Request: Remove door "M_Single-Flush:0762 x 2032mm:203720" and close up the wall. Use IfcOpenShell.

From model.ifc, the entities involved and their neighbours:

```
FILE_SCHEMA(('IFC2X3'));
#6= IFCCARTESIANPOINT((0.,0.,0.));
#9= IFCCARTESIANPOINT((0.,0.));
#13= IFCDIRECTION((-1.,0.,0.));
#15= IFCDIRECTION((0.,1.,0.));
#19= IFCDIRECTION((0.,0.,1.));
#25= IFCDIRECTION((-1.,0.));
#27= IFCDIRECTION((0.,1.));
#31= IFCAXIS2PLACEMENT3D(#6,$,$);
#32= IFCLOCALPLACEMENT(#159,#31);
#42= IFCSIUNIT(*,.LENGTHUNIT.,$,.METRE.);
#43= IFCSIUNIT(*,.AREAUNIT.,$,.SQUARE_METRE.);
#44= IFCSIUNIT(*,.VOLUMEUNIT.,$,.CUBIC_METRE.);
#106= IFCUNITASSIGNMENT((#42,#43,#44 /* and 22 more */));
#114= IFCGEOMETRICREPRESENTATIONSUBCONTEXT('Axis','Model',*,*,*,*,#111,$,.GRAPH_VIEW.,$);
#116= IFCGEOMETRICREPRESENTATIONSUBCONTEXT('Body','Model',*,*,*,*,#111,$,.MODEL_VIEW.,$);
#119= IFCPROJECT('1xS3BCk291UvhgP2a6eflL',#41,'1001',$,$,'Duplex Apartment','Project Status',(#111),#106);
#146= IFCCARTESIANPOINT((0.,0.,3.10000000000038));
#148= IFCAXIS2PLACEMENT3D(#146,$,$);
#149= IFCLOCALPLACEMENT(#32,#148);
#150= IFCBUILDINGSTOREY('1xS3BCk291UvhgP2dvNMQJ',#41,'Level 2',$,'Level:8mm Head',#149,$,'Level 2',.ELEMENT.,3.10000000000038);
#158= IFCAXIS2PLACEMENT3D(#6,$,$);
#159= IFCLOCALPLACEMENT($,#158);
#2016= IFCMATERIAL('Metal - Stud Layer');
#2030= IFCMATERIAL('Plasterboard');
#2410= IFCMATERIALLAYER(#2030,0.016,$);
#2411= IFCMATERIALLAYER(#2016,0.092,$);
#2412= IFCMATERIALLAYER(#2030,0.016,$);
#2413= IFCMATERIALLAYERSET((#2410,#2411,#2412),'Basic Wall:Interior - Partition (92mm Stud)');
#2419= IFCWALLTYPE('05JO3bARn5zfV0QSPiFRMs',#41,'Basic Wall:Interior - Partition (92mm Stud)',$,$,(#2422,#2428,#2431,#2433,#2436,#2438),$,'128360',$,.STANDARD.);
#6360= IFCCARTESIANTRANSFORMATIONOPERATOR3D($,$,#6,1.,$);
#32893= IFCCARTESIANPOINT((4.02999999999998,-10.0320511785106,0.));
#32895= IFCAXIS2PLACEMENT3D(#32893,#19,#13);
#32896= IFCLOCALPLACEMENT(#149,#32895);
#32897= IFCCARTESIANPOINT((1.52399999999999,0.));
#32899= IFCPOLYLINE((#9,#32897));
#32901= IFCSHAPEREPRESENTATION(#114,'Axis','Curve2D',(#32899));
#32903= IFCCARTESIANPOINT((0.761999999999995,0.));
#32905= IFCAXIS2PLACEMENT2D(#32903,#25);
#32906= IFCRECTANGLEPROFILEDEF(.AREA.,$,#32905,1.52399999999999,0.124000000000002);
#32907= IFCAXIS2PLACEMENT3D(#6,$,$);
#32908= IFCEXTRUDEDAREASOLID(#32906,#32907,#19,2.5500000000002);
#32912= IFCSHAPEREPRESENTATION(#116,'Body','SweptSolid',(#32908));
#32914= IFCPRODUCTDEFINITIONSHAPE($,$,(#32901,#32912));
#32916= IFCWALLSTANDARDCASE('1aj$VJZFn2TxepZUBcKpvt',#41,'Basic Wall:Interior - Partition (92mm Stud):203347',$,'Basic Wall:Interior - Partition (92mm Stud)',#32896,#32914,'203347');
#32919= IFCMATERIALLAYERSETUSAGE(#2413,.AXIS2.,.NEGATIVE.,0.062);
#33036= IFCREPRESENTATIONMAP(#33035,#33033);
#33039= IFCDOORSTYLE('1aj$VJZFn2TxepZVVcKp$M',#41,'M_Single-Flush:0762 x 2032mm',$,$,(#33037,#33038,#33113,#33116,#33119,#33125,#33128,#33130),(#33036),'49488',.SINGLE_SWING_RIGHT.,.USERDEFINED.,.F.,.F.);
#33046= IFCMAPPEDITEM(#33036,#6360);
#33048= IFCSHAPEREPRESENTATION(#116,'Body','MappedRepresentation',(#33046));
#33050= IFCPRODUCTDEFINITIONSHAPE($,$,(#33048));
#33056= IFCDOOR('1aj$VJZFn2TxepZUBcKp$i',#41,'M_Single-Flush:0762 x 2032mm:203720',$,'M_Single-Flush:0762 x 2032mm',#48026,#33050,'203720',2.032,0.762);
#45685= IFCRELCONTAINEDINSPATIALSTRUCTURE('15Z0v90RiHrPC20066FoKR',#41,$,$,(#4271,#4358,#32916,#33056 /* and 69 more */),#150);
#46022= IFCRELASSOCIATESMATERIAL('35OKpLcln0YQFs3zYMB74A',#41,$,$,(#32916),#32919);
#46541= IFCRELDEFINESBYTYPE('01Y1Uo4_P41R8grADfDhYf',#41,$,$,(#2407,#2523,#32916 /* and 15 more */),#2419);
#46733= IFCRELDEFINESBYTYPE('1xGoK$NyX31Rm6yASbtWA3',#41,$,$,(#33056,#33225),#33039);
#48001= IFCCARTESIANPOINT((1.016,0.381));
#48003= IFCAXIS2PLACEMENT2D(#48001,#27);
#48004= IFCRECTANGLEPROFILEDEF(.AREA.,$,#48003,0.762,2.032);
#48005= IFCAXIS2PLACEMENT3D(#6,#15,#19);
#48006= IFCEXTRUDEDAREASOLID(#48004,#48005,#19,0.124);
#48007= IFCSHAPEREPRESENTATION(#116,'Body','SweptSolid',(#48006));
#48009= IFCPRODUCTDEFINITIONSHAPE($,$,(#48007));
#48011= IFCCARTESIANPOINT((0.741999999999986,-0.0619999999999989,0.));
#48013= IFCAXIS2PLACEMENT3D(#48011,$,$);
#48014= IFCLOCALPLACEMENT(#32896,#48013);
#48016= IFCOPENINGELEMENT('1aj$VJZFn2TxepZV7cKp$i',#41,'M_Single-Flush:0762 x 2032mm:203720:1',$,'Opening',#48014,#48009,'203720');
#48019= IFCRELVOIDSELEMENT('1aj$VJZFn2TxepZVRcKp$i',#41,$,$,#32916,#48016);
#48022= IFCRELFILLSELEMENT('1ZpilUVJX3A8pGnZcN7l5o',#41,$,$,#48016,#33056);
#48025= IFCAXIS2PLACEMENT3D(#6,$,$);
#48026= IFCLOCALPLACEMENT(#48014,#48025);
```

```python
import ifcopenshell
import ifcopenshell.api.feature
import ifcopenshell.api.root
import ifcopenshell.geom
import ifcopenshell.util.shape

model = ifcopenshell.open("model.ifc")
settings = ifcopenshell.geom.settings()


def volume(element):
    """Net volume in cubic metres, openings subtracted."""
    shape = ifcopenshell.geom.create_shape(settings, element)
    return ifcopenshell.util.shape.get_volume(shape.geometry)


door = model.by_guid("1aj$VJZFn2TxepZUBcKp$i")
opening = door.FillsVoids[0].RelatingOpeningElement
wall = opening.VoidsElements[0].RelatingBuildingElement
before = volume(wall)

ifcopenshell.api.root.remove_product(model, product=door)
ifcopenshell.api.feature.remove_feature(model, feature=opening)

after = volume(wall)

print(f"wall volume {before:.3f} -> {after:.3f} m3")

model.write("model_v2.ifc")
```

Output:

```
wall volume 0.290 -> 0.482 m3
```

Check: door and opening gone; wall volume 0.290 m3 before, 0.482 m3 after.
